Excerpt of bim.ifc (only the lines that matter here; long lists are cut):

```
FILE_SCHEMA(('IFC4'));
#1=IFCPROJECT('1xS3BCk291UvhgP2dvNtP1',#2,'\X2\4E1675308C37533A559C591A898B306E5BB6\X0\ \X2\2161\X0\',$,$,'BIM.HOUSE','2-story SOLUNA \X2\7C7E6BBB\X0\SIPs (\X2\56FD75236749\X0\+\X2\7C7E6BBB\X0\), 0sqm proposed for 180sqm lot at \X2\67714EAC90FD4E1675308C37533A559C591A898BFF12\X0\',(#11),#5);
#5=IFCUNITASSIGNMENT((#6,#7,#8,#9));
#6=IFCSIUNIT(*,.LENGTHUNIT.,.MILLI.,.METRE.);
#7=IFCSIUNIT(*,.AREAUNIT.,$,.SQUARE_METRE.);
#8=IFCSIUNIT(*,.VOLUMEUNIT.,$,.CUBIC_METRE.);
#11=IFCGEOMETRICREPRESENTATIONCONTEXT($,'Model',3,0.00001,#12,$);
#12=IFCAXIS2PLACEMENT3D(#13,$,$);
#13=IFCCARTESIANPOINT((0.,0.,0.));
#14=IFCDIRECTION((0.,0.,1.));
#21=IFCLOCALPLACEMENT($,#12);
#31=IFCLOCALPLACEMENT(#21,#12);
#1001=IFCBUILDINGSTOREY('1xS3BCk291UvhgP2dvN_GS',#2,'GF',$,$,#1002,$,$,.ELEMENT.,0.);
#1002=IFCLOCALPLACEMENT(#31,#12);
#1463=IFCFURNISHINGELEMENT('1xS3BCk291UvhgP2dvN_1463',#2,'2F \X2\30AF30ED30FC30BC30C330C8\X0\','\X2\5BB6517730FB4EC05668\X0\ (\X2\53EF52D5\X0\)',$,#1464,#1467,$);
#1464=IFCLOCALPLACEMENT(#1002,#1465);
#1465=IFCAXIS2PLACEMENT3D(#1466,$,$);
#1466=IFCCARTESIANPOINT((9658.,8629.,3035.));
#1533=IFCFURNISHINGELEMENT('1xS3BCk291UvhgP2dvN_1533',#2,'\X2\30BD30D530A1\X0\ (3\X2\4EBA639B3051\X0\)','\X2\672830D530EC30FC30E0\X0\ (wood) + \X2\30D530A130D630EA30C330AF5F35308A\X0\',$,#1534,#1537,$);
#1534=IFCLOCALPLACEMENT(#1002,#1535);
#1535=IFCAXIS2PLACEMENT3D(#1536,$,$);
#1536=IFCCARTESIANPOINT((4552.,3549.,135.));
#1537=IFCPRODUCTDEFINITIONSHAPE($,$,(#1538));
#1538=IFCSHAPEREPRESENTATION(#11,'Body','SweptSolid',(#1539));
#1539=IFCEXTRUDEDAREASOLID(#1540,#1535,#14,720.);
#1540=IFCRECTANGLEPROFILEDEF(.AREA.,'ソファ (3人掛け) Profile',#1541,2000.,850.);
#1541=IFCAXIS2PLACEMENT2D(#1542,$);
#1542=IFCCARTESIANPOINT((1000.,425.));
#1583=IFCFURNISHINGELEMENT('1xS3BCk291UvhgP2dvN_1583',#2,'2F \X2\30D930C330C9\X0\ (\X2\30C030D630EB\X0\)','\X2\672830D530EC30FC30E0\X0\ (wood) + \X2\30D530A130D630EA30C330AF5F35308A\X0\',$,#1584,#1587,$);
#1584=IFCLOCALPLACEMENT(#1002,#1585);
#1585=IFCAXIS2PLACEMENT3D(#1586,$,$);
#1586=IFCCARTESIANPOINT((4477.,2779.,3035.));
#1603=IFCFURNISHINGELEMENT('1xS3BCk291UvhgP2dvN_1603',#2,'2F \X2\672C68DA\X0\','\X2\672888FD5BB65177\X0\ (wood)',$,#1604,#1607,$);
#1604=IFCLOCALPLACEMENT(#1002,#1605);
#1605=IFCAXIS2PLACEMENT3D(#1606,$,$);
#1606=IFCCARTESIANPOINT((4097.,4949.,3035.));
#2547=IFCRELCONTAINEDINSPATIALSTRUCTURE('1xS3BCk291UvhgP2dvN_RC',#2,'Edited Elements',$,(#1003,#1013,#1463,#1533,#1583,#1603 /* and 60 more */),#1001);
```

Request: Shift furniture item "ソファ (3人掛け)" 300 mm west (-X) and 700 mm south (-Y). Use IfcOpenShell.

```python
import ifcopenshell
import ifcopenshell.api.geometry
import ifcopenshell.util.placement
import ifcopenshell.util.unit

model = ifcopenshell.open("bim.ifc")
unit_scale = ifcopenshell.util.unit.calculate_unit_scale(model)

item = model.by_guid("1xS3BCk291UvhgP2dvN_1533")
matrix = ifcopenshell.util.placement.get_local_placement(item.ObjectPlacement)
matrix[0, 3] -= 0.3 / unit_scale
matrix[1, 3] -= 0.7 / unit_scale
ifcopenshell.api.geometry.edit_object_placement(model, product=item, matrix=matrix, is_si=False)

print(ifcopenshell.util.placement.get_local_placement(item.ObjectPlacement).round(3) + 0.0)

model.write("bim_edited.ifc")
```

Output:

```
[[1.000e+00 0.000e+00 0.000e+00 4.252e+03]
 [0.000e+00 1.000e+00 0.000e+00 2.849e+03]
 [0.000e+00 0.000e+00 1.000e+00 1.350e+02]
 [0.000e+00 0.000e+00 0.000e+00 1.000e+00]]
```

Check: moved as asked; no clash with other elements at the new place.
